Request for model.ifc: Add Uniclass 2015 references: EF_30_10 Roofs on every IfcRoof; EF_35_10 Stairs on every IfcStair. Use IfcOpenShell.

First a look at what the model holds.

```python
import ifcopenshell

model = ifcopenshell.open("model.ifc")
print(model.schema)
print("classifications:", [c.Name for c in model.by_type("IfcClassification")])
for ifc_class in ("IfcDoor", "IfcRoof", "IfcStair", "IfcWall", "IfcWindow"):
    print(ifc_class, len(model.by_type(ifc_class)))
```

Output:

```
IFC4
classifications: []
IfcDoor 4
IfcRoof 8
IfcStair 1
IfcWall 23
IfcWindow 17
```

```python
import ifcopenshell
import ifcopenshell.api.classification

model = ifcopenshell.open("model.ifc")

system = ifcopenshell.api.classification.add_classification(model, classification="Uniclass 2015")

codes = {
    "IfcRoof": ("EF_30_10", "Roofs"),
    "IfcStair": ("EF_35_10", "Stairs"),
}
for ifc_class, (code, name) in codes.items():
    products = model.by_type(ifc_class)
    ifcopenshell.api.classification.add_reference(
        model, products=products, classification=system, identification=code, name=name
    )
    print(code, len(products))

model.write("model-out.ifc")
```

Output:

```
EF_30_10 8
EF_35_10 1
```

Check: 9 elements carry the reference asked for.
